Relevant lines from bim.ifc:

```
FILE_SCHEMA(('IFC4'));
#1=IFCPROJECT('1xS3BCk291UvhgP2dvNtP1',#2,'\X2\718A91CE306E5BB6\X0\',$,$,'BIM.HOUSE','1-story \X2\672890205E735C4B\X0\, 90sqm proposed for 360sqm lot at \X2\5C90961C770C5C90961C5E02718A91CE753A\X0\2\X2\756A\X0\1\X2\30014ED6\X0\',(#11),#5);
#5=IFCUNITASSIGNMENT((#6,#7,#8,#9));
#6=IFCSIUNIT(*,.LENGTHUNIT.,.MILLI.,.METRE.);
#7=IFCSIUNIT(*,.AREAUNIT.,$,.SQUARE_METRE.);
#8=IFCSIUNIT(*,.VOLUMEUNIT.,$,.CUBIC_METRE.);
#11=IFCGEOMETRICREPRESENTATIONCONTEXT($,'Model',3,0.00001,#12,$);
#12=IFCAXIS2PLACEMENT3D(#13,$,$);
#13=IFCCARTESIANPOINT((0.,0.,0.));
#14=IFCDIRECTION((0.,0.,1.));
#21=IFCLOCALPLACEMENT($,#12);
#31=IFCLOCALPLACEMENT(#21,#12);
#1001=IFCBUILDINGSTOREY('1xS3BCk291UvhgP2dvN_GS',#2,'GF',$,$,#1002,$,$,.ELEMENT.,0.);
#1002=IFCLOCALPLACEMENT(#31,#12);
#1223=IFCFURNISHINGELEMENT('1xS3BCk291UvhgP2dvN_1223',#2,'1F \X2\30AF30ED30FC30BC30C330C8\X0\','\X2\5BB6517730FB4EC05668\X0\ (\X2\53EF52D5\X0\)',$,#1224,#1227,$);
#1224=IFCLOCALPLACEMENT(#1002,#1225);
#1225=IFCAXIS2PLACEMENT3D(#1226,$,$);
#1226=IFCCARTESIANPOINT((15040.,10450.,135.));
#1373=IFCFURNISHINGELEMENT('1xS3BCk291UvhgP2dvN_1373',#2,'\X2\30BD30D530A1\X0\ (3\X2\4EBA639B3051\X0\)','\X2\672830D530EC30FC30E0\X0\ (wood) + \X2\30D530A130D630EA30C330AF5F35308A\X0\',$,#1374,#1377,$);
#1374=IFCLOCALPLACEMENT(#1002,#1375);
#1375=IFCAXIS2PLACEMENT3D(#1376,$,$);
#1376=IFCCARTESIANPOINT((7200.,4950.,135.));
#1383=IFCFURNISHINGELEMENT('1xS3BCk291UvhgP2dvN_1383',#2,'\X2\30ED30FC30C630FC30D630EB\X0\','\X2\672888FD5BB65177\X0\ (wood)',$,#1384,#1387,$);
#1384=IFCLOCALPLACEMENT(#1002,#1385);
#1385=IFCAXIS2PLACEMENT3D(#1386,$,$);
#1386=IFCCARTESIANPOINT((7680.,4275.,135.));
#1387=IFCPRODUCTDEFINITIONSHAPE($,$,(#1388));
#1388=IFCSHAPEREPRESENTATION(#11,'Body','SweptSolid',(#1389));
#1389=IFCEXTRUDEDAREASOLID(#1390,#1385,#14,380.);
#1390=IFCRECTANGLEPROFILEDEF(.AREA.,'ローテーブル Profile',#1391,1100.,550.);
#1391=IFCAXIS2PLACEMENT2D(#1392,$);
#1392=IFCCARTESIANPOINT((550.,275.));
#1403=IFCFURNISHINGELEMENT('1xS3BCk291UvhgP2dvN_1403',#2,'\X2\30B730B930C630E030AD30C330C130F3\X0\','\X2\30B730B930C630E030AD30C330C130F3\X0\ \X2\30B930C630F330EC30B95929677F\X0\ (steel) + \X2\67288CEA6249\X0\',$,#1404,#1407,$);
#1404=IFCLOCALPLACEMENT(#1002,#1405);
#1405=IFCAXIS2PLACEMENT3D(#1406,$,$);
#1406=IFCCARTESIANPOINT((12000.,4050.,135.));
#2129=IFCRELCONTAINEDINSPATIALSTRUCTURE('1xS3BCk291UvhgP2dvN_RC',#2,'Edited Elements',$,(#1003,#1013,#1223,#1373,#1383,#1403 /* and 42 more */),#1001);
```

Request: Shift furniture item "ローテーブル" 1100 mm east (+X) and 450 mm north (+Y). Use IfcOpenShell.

```python
import ifcopenshell
import ifcopenshell.api.geometry
import ifcopenshell.util.placement
import ifcopenshell.util.unit

model = ifcopenshell.open("bim.ifc")
unit_scale = ifcopenshell.util.unit.calculate_unit_scale(model)

item = model.by_guid("1xS3BCk291UvhgP2dvN_1383")
matrix = ifcopenshell.util.placement.get_local_placement(item.ObjectPlacement)
matrix[0, 3] += 1.1 / unit_scale
matrix[1, 3] += 0.45 / unit_scale
ifcopenshell.api.geometry.edit_object_placement(model, product=item, matrix=matrix, is_si=False)

print(ifcopenshell.util.placement.get_local_placement(item.ObjectPlacement).round(3) + 0.0)

model.write("bim-out.ifc")
```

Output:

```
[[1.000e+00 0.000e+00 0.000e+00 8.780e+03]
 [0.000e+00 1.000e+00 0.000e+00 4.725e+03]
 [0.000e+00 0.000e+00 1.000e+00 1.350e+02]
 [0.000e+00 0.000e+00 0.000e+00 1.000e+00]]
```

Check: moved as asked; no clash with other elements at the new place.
